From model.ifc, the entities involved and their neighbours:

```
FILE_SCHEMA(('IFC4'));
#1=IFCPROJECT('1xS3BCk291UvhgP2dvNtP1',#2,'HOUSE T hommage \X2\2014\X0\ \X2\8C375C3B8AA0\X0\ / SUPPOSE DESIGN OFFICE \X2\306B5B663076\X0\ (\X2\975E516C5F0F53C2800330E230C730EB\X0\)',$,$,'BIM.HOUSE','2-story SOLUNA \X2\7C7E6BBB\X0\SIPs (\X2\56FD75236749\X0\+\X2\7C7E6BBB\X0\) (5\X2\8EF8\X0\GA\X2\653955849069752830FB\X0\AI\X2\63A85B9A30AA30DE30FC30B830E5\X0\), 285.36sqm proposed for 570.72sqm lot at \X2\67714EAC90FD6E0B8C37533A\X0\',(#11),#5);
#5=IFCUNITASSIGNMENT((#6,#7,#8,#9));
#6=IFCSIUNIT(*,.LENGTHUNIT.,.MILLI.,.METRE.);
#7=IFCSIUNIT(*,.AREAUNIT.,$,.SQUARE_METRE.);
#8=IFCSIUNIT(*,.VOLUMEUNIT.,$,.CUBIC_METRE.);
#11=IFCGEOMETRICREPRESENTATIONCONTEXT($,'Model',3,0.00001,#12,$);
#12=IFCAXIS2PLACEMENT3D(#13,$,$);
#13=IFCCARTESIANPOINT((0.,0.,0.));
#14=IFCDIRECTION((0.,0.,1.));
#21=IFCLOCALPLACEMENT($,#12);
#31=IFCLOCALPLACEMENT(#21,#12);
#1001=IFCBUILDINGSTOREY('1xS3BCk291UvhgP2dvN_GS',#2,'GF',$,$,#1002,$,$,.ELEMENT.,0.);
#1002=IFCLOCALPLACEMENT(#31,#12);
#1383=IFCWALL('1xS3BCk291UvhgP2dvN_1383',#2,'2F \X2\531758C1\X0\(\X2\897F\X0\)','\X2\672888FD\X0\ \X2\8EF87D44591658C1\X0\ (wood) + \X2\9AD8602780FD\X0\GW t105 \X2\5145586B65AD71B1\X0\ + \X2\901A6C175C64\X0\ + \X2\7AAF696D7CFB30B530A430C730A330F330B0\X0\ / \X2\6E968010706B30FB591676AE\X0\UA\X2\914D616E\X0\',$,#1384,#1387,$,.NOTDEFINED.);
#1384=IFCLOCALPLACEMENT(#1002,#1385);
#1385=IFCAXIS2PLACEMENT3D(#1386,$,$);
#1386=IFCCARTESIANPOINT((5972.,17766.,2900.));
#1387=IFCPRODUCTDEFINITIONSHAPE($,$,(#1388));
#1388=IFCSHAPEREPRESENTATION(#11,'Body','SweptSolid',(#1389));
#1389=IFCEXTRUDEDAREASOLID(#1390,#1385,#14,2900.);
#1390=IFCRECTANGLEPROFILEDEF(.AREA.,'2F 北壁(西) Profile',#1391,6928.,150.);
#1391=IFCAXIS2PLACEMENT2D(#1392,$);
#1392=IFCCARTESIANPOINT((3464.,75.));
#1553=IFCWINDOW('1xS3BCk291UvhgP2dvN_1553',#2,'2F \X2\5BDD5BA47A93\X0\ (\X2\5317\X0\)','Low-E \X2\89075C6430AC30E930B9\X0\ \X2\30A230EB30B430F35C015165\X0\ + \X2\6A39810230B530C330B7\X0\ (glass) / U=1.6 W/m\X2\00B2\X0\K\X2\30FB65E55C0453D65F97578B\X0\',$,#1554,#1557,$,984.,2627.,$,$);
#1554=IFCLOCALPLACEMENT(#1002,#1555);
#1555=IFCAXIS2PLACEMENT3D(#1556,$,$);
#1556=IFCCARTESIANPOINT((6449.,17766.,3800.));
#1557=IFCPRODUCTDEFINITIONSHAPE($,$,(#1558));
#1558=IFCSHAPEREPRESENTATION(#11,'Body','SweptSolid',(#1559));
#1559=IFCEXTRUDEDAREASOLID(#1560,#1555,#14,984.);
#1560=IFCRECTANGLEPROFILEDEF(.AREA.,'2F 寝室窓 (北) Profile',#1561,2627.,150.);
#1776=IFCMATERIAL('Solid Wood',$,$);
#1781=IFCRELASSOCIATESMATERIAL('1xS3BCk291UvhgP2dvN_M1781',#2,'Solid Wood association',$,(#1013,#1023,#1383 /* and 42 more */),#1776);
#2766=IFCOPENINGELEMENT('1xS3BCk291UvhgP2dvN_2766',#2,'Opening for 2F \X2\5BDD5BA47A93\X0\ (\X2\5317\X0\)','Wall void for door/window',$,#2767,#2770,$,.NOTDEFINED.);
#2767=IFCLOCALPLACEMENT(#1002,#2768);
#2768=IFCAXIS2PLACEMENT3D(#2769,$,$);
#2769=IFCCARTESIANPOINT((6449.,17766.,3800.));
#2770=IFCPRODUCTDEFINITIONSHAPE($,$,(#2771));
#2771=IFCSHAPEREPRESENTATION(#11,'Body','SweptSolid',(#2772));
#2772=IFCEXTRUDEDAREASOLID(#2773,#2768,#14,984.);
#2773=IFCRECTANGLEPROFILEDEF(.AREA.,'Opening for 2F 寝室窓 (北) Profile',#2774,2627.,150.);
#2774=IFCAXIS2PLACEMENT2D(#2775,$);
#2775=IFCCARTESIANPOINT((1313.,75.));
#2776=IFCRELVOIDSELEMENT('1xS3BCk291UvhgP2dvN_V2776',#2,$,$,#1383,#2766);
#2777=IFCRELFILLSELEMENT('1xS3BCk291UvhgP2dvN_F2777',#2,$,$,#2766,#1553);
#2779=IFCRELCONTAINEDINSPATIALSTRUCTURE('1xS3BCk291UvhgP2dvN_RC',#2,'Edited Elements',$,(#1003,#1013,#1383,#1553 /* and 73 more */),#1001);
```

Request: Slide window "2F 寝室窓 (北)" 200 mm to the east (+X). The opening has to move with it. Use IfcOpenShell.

```python
import ifcopenshell
import ifcopenshell.api.geometry
import ifcopenshell.util.placement
import ifcopenshell.util.unit

model = ifcopenshell.open("model.ifc")
unit_scale = ifcopenshell.util.unit.calculate_unit_scale(model)

window = model.by_id(1553)
opening = window.FillsVoids[0].RelatingOpeningElement
wall = opening.VoidsElements[0].RelatingBuildingElement

wall_matrix = ifcopenshell.util.placement.get_local_placement(wall.ObjectPlacement)
shift = wall_matrix[:3, 0] * 0.2 / unit_scale
before = ifcopenshell.util.placement.get_local_placement(window.ObjectPlacement)[:3, 3].copy()

# The window is not placed relative to its opening, so move both.
for product in (opening, window):
    matrix = ifcopenshell.util.placement.get_local_placement(product.ObjectPlacement)
    matrix[:3, 3] += shift
    ifcopenshell.api.geometry.edit_object_placement(model, product=product, matrix=matrix, is_si=False)

after = ifcopenshell.util.placement.get_local_placement(window.ObjectPlacement)[:3, 3]
print("window moved by", (after - before).round(3) + 0.0)

model.write("model_edited.ifc")
```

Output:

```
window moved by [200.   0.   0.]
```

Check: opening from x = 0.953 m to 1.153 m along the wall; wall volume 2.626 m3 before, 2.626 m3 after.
